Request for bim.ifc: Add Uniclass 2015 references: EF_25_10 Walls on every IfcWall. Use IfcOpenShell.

First a look at what the model holds.

```python
import ifcopenshell

model = ifcopenshell.open("bim.ifc")
print(model.schema)
print("classifications:", [c.Name for c in model.by_type("IfcClassification")])
for ifc_class in ("IfcDoor", "IfcRoof", "IfcStair", "IfcWall", "IfcWindow"):
    print(ifc_class, len(model.by_type(ifc_class)))
```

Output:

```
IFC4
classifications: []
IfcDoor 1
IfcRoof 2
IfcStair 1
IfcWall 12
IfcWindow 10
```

```python
import ifcopenshell
import ifcopenshell.api.classification

model = ifcopenshell.open("bim.ifc")

system = ifcopenshell.api.classification.add_classification(model, classification="Uniclass 2015")

codes = {
    "IfcWall": ("EF_25_10", "Walls"),
}
for ifc_class, (code, name) in codes.items():
    products = model.by_type(ifc_class)
    ifcopenshell.api.classification.add_reference(
        model, products=products, classification=system, identification=code, name=name
    )
    print(code, len(products))

model.write("bim_v2.ifc")
```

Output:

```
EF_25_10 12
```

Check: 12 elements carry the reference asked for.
